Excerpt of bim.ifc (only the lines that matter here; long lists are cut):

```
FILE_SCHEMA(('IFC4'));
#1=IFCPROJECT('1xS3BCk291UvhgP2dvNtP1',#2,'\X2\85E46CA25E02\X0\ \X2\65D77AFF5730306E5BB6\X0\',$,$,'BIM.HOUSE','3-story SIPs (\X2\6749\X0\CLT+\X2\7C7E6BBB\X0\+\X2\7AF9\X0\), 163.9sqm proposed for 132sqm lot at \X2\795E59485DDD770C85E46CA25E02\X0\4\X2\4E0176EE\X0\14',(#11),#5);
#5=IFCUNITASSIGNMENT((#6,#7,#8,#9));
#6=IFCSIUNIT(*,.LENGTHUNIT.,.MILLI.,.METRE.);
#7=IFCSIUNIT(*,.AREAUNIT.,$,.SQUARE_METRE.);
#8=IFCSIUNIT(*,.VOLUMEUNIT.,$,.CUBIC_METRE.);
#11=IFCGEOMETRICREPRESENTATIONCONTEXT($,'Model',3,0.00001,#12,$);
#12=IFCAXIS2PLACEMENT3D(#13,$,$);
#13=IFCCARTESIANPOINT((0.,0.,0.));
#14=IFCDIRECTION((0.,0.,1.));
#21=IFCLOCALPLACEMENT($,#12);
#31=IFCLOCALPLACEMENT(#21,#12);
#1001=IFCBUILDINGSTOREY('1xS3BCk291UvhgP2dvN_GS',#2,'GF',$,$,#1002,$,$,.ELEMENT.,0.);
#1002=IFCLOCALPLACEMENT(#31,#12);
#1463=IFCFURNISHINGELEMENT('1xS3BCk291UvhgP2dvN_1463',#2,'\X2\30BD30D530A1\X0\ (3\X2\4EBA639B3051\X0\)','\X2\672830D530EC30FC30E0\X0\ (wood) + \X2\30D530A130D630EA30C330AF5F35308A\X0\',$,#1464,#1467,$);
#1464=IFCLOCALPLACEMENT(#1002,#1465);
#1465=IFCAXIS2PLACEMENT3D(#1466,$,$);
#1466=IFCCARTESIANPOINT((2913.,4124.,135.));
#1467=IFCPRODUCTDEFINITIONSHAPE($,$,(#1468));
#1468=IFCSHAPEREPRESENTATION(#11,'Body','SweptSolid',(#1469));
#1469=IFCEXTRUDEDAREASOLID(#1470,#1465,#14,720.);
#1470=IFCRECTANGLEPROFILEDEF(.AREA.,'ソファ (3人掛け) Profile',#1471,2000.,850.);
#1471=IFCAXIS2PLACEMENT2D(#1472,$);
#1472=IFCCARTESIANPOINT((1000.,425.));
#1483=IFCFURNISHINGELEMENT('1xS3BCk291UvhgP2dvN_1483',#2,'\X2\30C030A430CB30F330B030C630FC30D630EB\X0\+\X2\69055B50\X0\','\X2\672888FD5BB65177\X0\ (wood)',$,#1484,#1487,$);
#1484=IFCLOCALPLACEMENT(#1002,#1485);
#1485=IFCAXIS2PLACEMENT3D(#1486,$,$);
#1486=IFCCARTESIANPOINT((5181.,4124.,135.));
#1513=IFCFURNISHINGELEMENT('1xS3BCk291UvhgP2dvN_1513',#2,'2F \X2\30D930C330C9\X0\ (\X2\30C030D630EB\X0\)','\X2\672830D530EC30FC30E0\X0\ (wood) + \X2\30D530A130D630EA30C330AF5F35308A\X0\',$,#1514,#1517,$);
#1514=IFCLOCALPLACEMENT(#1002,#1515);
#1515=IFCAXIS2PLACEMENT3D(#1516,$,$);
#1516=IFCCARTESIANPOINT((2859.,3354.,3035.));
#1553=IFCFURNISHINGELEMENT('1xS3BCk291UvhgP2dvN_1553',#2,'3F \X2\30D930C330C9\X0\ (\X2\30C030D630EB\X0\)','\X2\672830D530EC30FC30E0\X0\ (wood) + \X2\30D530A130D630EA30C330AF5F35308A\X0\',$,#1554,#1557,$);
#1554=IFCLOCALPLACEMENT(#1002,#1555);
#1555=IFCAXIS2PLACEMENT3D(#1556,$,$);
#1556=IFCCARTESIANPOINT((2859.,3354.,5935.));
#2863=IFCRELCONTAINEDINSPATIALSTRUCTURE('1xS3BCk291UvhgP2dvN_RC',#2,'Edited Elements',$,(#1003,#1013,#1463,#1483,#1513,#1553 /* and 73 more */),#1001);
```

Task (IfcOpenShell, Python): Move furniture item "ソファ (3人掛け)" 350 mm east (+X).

```python
import ifcopenshell
import ifcopenshell.api.geometry
import ifcopenshell.util.placement

model = ifcopenshell.open("bim.ifc")

item = model.by_guid("1xS3BCk291UvhgP2dvN_1463")
matrix = ifcopenshell.util.placement.get_local_placement(item.ObjectPlacement)
matrix[0, 3] += 350.0
ifcopenshell.api.geometry.edit_object_placement(model, product=item, matrix=matrix, is_si=False)

print(ifcopenshell.util.placement.get_local_placement(item.ObjectPlacement).round(3) + 0.0)

model.write("bim_updated.ifc")
```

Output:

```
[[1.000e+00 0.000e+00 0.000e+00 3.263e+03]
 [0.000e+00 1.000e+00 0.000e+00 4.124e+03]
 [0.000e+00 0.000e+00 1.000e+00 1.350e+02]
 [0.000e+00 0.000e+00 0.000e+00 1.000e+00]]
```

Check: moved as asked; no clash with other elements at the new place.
